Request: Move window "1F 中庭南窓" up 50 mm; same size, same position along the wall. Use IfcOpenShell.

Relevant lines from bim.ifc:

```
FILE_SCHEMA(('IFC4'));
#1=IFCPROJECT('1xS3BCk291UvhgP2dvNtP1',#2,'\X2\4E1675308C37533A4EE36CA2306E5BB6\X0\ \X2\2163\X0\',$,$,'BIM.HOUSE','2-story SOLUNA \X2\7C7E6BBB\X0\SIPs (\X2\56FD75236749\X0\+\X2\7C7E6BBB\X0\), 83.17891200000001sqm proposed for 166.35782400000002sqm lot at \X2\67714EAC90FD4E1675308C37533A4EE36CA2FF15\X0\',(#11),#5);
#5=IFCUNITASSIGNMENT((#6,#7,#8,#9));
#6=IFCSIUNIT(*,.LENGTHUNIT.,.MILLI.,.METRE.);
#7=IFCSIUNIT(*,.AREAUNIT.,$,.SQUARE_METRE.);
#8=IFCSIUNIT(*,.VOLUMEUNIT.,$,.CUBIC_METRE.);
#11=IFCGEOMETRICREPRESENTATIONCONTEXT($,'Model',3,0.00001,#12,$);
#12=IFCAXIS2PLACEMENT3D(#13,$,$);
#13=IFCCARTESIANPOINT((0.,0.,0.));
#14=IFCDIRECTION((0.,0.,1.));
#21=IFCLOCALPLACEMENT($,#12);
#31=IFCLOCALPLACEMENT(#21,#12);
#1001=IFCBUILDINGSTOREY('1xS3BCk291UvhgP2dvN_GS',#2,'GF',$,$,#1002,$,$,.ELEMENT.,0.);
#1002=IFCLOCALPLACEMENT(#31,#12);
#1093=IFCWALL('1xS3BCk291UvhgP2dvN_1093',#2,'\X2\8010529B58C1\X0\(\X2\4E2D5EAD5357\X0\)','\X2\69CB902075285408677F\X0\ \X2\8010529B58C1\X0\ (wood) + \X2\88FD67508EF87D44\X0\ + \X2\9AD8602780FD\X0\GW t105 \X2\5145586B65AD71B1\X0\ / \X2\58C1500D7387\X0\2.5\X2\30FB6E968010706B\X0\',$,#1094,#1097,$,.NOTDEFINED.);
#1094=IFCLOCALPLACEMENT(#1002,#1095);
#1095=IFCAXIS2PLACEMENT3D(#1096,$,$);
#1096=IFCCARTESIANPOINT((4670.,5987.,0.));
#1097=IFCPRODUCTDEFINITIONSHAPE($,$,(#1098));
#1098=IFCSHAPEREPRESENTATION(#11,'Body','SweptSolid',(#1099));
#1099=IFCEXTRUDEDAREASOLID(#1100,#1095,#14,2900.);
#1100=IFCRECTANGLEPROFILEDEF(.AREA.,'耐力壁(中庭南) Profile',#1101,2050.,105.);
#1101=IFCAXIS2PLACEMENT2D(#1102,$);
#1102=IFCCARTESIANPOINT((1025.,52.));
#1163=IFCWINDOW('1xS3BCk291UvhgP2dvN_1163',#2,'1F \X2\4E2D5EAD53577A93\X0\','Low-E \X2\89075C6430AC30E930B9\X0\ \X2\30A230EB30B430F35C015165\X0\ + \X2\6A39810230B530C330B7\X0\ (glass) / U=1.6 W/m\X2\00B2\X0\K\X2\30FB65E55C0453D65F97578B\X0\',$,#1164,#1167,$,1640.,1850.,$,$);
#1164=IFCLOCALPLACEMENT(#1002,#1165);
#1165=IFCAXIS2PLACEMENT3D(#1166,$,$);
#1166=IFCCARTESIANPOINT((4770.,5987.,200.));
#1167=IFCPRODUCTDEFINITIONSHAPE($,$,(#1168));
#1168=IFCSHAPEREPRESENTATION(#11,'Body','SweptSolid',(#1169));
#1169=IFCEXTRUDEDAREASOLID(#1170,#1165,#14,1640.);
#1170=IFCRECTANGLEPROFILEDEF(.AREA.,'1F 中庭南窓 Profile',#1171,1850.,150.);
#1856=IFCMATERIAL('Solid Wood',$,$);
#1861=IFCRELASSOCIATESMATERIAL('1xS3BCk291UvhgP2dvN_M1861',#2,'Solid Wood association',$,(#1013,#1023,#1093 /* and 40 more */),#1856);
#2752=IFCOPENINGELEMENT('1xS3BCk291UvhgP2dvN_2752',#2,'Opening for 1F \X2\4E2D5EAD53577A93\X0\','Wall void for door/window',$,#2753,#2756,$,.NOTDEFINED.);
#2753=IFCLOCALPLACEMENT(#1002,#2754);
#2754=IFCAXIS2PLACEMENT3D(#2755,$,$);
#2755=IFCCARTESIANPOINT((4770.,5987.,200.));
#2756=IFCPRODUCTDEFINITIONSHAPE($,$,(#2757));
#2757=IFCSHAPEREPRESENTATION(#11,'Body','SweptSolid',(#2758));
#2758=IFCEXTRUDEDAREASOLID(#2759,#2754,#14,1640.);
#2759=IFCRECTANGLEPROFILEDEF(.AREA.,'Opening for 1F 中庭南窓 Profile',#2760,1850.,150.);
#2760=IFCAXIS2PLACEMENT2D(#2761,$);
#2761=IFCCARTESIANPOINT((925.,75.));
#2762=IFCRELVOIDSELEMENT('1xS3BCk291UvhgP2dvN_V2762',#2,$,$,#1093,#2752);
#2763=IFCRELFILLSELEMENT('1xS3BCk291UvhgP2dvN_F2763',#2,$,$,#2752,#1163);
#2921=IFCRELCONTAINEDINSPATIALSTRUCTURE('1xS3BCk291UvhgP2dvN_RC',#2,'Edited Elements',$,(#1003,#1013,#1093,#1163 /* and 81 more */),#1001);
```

```python
import numpy as np
import ifcopenshell
import ifcopenshell.api.geometry
import ifcopenshell.util.placement
import ifcopenshell.util.unit

model = ifcopenshell.open("bim.ifc")
unit_scale = ifcopenshell.util.unit.calculate_unit_scale(model)

window = model.by_guid("1xS3BCk291UvhgP2dvN_1163")
opening = window.FillsVoids[0].RelatingOpeningElement
dz = 0.05 / unit_scale

shift = np.array([0.0, 0.0, dz])
# The window is not placed relative to its opening, so move both.
for product in (opening, window):
    matrix = ifcopenshell.util.placement.get_local_placement(product.ObjectPlacement)
    matrix[:3, 3] += shift
    ifcopenshell.api.geometry.edit_object_placement(model, product=product, matrix=matrix, is_si=False)

print(f"moved by {dz * unit_scale:+.3f} m")

model.write("bim_edited.ifc")
```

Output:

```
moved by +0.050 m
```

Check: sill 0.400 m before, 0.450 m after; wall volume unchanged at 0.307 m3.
